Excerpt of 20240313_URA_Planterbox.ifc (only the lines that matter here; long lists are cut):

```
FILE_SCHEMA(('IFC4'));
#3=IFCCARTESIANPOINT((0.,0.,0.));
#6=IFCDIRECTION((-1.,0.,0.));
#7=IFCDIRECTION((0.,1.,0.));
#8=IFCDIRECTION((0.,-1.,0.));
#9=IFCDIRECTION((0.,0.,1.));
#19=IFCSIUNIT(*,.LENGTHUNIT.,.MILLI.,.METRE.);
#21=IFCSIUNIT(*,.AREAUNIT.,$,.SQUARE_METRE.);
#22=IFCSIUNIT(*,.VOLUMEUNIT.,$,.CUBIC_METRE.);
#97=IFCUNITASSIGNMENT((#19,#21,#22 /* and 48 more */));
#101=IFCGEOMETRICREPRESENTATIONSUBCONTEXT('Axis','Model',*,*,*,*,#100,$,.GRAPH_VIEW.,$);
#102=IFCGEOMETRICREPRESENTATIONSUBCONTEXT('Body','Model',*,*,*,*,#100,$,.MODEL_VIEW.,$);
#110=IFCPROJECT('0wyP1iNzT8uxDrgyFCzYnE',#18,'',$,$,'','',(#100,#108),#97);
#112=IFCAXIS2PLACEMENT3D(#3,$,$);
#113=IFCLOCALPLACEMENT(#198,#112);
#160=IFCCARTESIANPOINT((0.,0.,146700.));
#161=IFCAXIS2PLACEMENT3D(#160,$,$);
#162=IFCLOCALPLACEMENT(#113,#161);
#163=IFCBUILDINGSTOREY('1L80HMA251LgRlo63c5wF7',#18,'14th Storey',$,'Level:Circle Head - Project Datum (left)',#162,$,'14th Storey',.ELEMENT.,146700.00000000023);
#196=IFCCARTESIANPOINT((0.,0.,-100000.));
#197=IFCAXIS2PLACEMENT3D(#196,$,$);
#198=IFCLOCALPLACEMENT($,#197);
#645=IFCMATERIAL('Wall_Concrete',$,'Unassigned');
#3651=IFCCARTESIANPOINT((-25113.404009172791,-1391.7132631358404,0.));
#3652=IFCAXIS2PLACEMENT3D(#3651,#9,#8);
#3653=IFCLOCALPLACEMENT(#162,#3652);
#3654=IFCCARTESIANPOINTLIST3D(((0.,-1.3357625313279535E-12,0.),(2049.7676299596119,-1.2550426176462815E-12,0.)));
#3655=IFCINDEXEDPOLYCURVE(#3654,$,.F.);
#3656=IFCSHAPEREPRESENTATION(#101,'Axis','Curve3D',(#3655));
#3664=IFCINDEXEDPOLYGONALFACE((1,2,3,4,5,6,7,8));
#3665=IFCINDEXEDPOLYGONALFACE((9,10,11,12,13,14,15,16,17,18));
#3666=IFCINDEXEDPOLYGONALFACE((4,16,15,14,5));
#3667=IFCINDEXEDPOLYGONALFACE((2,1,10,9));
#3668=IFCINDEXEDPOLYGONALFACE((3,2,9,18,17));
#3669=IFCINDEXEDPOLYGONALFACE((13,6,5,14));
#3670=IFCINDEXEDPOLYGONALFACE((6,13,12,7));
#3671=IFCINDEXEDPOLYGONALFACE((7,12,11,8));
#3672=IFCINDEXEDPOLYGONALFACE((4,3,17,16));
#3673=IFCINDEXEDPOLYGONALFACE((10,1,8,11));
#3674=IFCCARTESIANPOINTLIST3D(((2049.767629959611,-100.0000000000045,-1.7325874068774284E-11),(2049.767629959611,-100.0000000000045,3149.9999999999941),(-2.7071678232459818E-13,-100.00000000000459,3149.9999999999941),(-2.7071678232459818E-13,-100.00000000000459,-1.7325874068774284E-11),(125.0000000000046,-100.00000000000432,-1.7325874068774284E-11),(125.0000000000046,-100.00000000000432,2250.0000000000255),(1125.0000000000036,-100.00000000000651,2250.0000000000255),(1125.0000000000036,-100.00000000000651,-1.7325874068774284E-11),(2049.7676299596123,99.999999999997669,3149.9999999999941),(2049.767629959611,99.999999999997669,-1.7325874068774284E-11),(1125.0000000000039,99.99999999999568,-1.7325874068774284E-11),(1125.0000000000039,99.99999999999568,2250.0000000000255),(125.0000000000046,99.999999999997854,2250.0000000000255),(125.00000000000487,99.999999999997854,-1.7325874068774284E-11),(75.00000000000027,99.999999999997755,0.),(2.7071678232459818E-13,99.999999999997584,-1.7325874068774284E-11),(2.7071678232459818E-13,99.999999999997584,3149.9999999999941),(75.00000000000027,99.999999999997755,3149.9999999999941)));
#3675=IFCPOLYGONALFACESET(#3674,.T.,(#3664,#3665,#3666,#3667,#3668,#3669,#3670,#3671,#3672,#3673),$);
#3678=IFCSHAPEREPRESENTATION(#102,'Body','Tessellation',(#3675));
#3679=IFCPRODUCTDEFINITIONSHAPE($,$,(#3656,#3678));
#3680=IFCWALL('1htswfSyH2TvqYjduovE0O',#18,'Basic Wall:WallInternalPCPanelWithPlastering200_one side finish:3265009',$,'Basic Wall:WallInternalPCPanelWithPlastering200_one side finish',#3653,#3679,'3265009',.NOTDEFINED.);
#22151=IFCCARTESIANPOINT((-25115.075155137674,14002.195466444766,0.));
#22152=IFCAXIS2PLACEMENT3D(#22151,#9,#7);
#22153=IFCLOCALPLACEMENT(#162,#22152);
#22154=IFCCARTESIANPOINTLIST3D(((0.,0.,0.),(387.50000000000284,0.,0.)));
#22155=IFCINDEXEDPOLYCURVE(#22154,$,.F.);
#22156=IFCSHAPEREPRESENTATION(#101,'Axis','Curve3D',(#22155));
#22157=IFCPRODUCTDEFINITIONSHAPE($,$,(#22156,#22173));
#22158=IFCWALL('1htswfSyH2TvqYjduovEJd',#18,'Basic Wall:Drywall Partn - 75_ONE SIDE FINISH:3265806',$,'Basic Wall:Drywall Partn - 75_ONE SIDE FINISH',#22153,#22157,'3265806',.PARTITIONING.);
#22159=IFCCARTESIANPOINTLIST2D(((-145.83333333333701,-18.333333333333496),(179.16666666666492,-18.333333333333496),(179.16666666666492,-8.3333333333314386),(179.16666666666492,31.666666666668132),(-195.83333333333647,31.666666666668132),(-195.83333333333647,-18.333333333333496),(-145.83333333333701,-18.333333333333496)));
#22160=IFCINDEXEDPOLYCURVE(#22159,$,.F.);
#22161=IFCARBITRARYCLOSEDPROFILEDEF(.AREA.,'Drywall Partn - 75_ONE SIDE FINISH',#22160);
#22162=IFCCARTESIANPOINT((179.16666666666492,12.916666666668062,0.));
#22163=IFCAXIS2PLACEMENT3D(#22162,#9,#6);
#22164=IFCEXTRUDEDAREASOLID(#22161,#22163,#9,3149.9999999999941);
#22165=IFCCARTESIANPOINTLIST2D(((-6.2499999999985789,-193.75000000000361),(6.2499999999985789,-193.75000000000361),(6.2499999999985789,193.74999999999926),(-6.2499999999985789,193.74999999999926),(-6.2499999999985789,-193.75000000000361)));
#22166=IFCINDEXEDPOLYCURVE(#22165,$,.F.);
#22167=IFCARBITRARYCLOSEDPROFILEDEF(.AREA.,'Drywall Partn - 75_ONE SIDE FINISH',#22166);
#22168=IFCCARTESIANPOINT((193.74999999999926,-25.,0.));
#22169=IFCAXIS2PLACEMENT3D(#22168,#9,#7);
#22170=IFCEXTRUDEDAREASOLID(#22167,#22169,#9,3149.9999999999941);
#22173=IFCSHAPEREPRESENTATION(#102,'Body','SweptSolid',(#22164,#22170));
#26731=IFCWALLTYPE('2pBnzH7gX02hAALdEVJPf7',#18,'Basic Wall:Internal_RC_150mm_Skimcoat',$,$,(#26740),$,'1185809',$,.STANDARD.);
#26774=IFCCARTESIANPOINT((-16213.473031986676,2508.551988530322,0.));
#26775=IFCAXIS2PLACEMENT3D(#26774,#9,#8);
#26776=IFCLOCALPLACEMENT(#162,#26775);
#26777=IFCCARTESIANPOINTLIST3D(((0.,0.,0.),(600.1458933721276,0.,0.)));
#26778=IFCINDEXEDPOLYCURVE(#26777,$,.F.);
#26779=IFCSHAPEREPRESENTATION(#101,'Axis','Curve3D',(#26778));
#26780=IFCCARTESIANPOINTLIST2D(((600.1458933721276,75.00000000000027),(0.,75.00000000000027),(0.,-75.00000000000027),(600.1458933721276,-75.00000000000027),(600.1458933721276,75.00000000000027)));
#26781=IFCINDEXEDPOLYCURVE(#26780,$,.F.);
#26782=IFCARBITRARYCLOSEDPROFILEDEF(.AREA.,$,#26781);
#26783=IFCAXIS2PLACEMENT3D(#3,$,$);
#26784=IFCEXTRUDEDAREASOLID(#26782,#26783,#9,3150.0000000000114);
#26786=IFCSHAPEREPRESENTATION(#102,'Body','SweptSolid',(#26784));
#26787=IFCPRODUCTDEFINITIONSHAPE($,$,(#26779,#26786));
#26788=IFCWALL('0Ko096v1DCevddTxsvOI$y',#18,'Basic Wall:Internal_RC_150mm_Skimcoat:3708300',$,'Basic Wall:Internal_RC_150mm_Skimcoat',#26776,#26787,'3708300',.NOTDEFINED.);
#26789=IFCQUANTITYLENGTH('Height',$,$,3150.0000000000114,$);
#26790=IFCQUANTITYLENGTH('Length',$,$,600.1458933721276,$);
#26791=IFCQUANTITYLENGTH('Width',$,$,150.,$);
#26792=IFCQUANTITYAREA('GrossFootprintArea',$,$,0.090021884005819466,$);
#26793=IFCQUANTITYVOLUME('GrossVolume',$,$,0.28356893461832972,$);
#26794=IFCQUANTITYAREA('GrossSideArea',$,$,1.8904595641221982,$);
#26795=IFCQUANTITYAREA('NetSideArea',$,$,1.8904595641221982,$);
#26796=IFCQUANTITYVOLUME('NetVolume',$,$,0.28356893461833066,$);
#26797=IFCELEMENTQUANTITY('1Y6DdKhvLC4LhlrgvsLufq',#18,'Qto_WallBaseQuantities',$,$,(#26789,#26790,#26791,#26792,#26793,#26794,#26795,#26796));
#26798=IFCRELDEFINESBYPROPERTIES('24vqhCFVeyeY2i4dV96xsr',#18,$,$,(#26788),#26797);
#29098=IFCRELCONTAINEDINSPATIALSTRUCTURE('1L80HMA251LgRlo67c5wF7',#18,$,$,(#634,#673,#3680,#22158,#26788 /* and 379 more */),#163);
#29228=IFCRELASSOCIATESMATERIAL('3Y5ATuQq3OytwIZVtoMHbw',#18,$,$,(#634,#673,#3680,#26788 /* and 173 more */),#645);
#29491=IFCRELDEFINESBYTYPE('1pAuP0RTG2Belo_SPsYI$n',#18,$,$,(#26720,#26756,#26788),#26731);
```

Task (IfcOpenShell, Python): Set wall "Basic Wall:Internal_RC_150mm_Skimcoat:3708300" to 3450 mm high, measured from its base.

```python
import ifcopenshell
import ifcopenshell.api.pset
import ifcopenshell.geom
import ifcopenshell.util.element
import ifcopenshell.util.representation
import ifcopenshell.util.shape
import ifcopenshell.util.unit

model = ifcopenshell.open("20240313_URA_Planterbox.ifc")
unit_scale = ifcopenshell.util.unit.calculate_unit_scale(model)
area_scale = ifcopenshell.util.unit.calculate_unit_scale(model, "AREAUNIT")
volume_scale = ifcopenshell.util.unit.calculate_unit_scale(model, "VOLUMEUNIT")
settings = ifcopenshell.geom.settings()


def volume(element):
    """Net volume in cubic metres, openings subtracted."""
    shape = ifcopenshell.geom.create_shape(settings, element)
    return ifcopenshell.util.shape.get_volume(shape.geometry)


wall = model.by_guid("0Ko096v1DCevddTxsvOI$y")
before = volume(wall)

body = ifcopenshell.util.representation.get_representation(wall, "Model", "Body")
solid = body.Items[0]
old_height = solid.Depth
solid.Depth = 3450.0
after = volume(wall)
thickness = 0.15  # wall thickness in metres

# Update the stored height, areas and volumes.
qto = model.by_id(ifcopenshell.util.element.get_pset(wall, "Qto_WallBaseQuantities", should_inherit=False)["id"])
ifcopenshell.api.pset.edit_qto(model, qto=qto, properties={
    "Height": solid.Depth,
    "GrossVolume": ifcopenshell.util.element.get_pset(wall, "Qto_WallBaseQuantities", "GrossVolume") * solid.Depth / old_height,
    "GrossSideArea": ifcopenshell.util.element.get_pset(wall, "Qto_WallBaseQuantities", "GrossSideArea") * solid.Depth / old_height,
    "NetSideArea": after / thickness / area_scale,
    "NetVolume": after / volume_scale,
})

print(f"height {old_height:g} -> {solid.Depth:g}, volume {before:.3f} -> {after:.3f} m3")

model.write("20240313_URA_Planterbox-out.ifc")
```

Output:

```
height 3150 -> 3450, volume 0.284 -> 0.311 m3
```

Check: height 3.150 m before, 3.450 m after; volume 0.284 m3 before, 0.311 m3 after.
